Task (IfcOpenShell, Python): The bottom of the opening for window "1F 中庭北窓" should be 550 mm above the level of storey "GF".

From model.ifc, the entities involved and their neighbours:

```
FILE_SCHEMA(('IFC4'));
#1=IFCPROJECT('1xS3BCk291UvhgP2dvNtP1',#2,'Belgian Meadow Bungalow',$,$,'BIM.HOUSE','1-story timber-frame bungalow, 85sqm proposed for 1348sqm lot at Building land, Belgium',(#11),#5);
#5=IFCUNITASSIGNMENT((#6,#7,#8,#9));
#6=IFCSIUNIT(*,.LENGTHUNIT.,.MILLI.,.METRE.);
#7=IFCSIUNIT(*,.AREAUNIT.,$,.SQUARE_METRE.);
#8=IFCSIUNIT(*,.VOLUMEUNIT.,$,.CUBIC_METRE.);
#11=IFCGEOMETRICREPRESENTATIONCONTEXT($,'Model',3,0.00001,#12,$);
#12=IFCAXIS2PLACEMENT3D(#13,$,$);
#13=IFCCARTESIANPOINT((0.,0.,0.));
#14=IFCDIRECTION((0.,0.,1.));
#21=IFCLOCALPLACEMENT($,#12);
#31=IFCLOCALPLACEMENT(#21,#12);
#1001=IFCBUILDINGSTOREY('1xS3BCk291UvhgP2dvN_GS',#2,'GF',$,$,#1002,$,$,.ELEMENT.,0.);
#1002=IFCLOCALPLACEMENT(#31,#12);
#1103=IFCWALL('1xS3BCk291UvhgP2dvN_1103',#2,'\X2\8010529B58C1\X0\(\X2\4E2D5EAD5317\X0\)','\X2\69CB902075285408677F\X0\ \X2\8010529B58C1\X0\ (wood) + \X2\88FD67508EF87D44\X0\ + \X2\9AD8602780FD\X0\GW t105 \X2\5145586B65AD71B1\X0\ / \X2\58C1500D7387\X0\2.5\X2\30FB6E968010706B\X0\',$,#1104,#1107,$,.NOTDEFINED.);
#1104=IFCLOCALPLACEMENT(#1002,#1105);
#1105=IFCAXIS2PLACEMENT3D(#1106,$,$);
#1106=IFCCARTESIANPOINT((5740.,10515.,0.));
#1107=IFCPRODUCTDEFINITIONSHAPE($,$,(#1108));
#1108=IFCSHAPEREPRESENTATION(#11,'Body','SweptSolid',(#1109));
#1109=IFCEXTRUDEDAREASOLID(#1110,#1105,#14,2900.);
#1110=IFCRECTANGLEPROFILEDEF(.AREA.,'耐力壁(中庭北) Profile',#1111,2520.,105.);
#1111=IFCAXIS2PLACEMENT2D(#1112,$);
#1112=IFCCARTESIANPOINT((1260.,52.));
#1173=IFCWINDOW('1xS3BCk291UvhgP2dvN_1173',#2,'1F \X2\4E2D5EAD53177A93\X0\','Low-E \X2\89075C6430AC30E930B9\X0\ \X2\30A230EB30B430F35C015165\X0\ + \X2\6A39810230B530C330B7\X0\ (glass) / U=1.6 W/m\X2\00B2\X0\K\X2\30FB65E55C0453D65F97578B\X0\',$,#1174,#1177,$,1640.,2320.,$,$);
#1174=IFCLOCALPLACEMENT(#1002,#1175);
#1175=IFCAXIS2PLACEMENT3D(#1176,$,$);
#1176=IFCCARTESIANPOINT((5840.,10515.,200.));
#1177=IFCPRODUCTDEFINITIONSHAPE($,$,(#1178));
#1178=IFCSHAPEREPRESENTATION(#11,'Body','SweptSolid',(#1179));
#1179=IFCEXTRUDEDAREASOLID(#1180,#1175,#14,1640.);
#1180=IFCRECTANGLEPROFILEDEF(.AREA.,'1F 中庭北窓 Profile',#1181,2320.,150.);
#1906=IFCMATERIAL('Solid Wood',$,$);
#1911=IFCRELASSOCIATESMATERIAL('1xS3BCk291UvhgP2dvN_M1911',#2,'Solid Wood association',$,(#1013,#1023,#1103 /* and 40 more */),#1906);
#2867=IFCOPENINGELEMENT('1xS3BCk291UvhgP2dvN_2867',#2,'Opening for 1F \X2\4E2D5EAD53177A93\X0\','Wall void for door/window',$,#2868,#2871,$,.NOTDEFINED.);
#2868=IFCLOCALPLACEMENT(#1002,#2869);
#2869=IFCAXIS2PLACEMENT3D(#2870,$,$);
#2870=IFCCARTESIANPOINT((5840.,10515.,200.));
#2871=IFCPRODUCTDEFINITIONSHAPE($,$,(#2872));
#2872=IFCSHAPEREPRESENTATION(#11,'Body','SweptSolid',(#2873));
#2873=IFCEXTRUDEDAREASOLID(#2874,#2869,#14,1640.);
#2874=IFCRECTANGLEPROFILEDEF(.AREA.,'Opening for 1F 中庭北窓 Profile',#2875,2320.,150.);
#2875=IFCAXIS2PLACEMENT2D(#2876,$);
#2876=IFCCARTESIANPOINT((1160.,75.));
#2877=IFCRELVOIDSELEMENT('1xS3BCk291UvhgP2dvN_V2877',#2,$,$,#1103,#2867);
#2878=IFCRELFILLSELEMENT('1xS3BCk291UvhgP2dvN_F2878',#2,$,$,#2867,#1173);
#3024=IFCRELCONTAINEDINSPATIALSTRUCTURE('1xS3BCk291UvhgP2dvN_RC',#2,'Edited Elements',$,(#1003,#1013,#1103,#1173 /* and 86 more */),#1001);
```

```python
import numpy as np
import ifcopenshell
import ifcopenshell.api.geometry
import ifcopenshell.geom
import ifcopenshell.util.element
import ifcopenshell.util.placement
import ifcopenshell.util.shape
import ifcopenshell.util.unit

model = ifcopenshell.open("model.ifc")
unit_scale = ifcopenshell.util.unit.calculate_unit_scale(model)

window = model.by_guid("1xS3BCk291UvhgP2dvN_1173")
opening = window.FillsVoids[0].RelatingOpeningElement
storey = ifcopenshell.util.element.get_container(window, ifc_class="IfcBuildingStorey")
level = ifcopenshell.util.placement.get_local_placement(storey.ObjectPlacement)[2, 3]

# The opening's origin need not be at the sill, so measure its lowest point.
shape = ifcopenshell.geom.create_shape(ifcopenshell.geom.settings(), opening)
bottom = ifcopenshell.util.shape.get_shape_bottom_elevation(shape, shape.geometry) / unit_scale
dz = level + 550.0 - bottom

shift = np.array([0.0, 0.0, dz])
# The window is not placed relative to its opening, so move both.
for product in (opening, window):
    matrix = ifcopenshell.util.placement.get_local_placement(product.ObjectPlacement)
    matrix[:3, 3] += shift
    ifcopenshell.api.geometry.edit_object_placement(model, product=product, matrix=matrix, is_si=False)

print(f"moved by {dz * unit_scale:+.3f} m")

model.write("model_rev.ifc")
```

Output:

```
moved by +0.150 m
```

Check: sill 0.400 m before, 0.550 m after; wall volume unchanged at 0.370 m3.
